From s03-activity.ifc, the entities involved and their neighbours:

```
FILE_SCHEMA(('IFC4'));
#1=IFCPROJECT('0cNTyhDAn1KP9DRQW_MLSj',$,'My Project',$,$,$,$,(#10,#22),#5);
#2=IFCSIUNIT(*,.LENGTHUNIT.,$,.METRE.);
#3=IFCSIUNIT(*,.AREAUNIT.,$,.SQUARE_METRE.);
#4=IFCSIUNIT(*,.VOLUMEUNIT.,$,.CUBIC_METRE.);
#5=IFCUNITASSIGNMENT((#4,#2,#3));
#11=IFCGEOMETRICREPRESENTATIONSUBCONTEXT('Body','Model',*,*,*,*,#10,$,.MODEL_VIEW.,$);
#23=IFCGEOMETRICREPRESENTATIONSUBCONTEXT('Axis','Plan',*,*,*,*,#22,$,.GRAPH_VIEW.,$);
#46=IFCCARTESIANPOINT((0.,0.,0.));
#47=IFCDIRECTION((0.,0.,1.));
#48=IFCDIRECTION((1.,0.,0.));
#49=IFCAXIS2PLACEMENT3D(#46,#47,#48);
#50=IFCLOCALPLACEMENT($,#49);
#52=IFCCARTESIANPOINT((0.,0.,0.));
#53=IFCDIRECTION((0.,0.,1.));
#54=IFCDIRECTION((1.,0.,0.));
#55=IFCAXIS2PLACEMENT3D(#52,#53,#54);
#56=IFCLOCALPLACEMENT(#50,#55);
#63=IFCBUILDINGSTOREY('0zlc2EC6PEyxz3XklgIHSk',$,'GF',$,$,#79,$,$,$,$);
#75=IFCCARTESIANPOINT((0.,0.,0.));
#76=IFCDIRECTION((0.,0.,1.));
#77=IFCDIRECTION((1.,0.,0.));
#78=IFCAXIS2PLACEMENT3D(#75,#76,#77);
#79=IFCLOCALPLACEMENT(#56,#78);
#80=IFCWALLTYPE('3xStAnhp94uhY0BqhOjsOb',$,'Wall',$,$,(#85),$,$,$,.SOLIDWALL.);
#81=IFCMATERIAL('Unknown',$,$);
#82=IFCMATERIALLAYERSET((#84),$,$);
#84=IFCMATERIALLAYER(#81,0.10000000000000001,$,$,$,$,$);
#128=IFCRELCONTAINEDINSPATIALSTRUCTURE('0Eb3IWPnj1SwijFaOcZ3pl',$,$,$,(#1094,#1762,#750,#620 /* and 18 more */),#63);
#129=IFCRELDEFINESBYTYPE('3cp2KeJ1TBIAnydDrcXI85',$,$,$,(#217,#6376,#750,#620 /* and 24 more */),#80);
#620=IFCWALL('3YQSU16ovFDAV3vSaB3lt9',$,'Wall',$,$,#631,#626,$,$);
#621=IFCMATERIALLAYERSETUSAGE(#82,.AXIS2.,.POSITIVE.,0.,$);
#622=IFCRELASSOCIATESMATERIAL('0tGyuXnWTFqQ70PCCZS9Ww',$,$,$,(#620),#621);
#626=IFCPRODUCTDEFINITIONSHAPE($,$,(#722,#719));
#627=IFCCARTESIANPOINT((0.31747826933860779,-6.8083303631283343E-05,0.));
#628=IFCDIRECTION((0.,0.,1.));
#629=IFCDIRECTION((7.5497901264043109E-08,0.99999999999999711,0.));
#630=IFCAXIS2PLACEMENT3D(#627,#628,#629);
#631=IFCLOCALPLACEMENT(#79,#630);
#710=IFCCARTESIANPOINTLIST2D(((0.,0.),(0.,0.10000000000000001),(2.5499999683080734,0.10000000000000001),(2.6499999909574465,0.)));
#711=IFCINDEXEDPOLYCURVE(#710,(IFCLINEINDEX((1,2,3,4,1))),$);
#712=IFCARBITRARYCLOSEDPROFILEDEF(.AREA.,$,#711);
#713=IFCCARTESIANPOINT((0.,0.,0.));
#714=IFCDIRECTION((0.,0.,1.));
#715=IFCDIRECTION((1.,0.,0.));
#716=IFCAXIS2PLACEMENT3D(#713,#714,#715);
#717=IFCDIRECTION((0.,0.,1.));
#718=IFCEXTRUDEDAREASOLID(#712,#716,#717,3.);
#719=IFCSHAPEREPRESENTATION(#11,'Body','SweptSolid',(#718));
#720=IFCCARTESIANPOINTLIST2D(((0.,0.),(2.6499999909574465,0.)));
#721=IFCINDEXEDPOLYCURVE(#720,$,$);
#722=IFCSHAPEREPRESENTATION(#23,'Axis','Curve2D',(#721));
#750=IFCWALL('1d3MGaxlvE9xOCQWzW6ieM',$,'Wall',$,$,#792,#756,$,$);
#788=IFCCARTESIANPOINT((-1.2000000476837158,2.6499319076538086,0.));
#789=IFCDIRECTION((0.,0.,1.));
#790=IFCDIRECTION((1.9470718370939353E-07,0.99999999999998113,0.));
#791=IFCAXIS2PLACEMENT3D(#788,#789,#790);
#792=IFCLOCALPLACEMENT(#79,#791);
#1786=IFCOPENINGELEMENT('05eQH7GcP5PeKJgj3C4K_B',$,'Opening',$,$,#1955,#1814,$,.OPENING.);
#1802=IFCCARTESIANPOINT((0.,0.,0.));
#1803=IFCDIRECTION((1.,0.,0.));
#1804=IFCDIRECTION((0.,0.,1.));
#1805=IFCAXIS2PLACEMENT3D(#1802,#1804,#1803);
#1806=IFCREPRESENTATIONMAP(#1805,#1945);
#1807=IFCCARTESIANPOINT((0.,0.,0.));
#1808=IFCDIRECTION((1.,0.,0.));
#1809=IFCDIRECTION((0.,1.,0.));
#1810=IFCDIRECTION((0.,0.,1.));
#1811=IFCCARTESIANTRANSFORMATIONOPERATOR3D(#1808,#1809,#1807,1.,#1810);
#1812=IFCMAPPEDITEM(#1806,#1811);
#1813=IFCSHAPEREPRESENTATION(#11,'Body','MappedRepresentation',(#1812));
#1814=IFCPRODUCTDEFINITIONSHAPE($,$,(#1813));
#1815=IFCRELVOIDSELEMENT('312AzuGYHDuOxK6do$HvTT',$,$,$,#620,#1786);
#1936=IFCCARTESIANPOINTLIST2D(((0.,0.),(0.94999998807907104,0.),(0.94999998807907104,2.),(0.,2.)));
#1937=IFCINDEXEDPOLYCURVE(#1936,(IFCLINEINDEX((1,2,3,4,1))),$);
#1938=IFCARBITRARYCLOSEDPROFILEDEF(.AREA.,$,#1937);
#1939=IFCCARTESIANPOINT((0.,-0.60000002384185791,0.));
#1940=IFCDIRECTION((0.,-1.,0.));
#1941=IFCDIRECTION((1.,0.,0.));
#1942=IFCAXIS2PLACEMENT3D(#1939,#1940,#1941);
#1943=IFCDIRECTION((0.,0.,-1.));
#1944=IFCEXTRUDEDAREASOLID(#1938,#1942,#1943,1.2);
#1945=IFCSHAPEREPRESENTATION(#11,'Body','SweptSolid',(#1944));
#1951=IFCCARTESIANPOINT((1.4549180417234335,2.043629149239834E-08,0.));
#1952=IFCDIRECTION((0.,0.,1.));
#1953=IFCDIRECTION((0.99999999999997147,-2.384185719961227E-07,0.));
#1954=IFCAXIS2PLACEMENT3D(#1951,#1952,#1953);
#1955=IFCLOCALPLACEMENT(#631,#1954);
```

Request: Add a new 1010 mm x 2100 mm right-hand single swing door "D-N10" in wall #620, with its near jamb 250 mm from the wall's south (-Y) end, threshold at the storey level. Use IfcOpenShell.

```python
import numpy as np
import ifcopenshell
import ifcopenshell.api.feature
import ifcopenshell.api.geometry
import ifcopenshell.api.root
import ifcopenshell.api.spatial
import ifcopenshell.geom
import ifcopenshell.util.element
import ifcopenshell.util.placement
import ifcopenshell.util.representation
import ifcopenshell.util.shape
import ifcopenshell.util.unit

model = ifcopenshell.open("s03-activity.ifc")
unit_scale = ifcopenshell.util.unit.calculate_unit_scale(model)
settings = ifcopenshell.geom.settings()


def volume(element):
    """Net volume in cubic metres, openings subtracted."""
    shape = ifcopenshell.geom.create_shape(settings, element)
    return ifcopenshell.util.shape.get_volume(shape.geometry)


wall = model.by_guid("3YQSU16ovFDAV3vSaB3lt9")
storey = ifcopenshell.util.element.get_container(wall, ifc_class="IfcBuildingStorey")
context = ifcopenshell.util.representation.get_context(model, "Model", "Body", "MODEL_VIEW")
before = volume(wall)

width, height, from_end, sill = 1.01, 2.1, 0.25, 0.0  # metres

# The wall runs along its own X axis, and the end named is its -X end.
wall_shape = ifcopenshell.geom.create_shape(settings, wall)
x, y, z = ifcopenshell.util.shape.get_vertices(wall_shape.geometry).T
start = x.min() + from_end
face, thickness = float(y.min()), float(y.max() - y.min())
wall_matrix = ifcopenshell.util.placement.get_local_placement(wall.ObjectPlacement)
level = ifcopenshell.util.placement.get_local_placement(storey.ObjectPlacement)[2, 3]


def in_wall(x, y):
    """Placement at x, y metres in the wall's axes, at sill height."""
    matrix = wall_matrix.copy()
    matrix[:, 3] = wall_matrix @ np.array([x / unit_scale, y / unit_scale, 0.0, 1.0])
    matrix[2, 3] = level + sill / unit_scale
    return matrix


# Opening: a box that overshoots both wall faces by 50 mm.
opening = ifcopenshell.api.root.create_entity(model, ifc_class="IfcOpeningElement", predefined_type="OPENING")
box = ifcopenshell.api.geometry.add_wall_representation(
    model, context=context, length=width, height=height, thickness=thickness + 0.1
)
ifcopenshell.api.geometry.assign_representation(model, product=opening, representation=box)
ifcopenshell.api.geometry.edit_object_placement(model, product=opening, matrix=in_wall(start, face - 0.05), is_si=False)
ifcopenshell.api.feature.add_feature(model, feature=opening, element=wall)

door = ifcopenshell.api.root.create_entity(model, ifc_class="IfcDoor", name="D-N10", predefined_type="DOOR")
door.OverallWidth, door.OverallHeight = width / unit_scale, height / unit_scale
door.OperationType = "SINGLE_SWING_RIGHT"
body = ifcopenshell.api.geometry.add_door_representation(
    model,
    context=context,
    overall_width=door.OverallWidth,
    overall_height=door.OverallHeight,
    operation_type="SINGLE_SWING_RIGHT",
    lining_properties={"LiningDepth": thickness / unit_scale, "ThresholdDepth": thickness / unit_scale},
)
ifcopenshell.api.geometry.assign_representation(model, product=door, representation=body)
ifcopenshell.api.spatial.assign_container(model, products=[door], relating_structure=storey)
ifcopenshell.api.feature.add_filling(model, opening=opening, element=door)

# The lining spans the wall, so the door starts at the wall face.
ifcopenshell.api.geometry.edit_object_placement(model, product=door, matrix=in_wall(start, face), is_si=False)

after = volume(wall)

print(f"wall volume {before:.3f} -> {after:.3f} m3")

model.write("s03-activity_edited.ifc")
```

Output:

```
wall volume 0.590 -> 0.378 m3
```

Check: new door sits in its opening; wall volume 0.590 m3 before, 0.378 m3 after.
